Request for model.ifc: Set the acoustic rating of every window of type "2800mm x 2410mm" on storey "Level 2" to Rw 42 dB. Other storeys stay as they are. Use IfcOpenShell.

First a look at what the model holds.

```python
import ifcopenshell
import ifcopenshell.util.element

model = ifcopenshell.open("model.ifc")
print(model.schema)
storey = next(s for s in model.by_type("IfcBuildingStorey") if s.Name == "Level 2")
windows = [e for e in ifcopenshell.util.element.get_decomposition(storey) if e.is_a("IfcWindow")]
seen = {}
for e in windows:
    element_type = ifcopenshell.util.element.get_type(e)
    key = (element_type.Name if element_type != e and element_type else None, ifcopenshell.util.element.get_pset(e, "Pset_WindowCommon", "AcousticRating"))
    seen[key] = seen.get(key, 0) + 1
for (name, value), count in sorted(seen.items(), key=str):
    print(count, "x", name, "|", value)
```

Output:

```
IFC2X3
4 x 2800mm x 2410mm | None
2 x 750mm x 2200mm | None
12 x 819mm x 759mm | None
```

```python
import ifcopenshell
import ifcopenshell.api.pset
import ifcopenshell.util.element

model = ifcopenshell.open("model.ifc")

storey = next(s for s in model.by_type("IfcBuildingStorey") if s.Name == "Level 2")
windows = [e for e in ifcopenshell.util.element.get_decomposition(storey) if e.is_a("IfcWindow")]

count = 0
for e in windows:
    element_type = ifcopenshell.util.element.get_type(e)
    if element_type in (None, e) or element_type.Name != "2800mm x 2410mm":
        continue
    # add_pset returns the element's existing set when there is one.
    pset = ifcopenshell.api.pset.add_pset(model, product=e, name="Pset_WindowCommon")
    ifcopenshell.api.pset.edit_pset(model, pset=pset, properties={"AcousticRating": "Rw 42 dB"})
    count += 1

print(count, "windows updated")

model.write("model_v2.ifc")
```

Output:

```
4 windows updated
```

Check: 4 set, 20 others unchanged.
